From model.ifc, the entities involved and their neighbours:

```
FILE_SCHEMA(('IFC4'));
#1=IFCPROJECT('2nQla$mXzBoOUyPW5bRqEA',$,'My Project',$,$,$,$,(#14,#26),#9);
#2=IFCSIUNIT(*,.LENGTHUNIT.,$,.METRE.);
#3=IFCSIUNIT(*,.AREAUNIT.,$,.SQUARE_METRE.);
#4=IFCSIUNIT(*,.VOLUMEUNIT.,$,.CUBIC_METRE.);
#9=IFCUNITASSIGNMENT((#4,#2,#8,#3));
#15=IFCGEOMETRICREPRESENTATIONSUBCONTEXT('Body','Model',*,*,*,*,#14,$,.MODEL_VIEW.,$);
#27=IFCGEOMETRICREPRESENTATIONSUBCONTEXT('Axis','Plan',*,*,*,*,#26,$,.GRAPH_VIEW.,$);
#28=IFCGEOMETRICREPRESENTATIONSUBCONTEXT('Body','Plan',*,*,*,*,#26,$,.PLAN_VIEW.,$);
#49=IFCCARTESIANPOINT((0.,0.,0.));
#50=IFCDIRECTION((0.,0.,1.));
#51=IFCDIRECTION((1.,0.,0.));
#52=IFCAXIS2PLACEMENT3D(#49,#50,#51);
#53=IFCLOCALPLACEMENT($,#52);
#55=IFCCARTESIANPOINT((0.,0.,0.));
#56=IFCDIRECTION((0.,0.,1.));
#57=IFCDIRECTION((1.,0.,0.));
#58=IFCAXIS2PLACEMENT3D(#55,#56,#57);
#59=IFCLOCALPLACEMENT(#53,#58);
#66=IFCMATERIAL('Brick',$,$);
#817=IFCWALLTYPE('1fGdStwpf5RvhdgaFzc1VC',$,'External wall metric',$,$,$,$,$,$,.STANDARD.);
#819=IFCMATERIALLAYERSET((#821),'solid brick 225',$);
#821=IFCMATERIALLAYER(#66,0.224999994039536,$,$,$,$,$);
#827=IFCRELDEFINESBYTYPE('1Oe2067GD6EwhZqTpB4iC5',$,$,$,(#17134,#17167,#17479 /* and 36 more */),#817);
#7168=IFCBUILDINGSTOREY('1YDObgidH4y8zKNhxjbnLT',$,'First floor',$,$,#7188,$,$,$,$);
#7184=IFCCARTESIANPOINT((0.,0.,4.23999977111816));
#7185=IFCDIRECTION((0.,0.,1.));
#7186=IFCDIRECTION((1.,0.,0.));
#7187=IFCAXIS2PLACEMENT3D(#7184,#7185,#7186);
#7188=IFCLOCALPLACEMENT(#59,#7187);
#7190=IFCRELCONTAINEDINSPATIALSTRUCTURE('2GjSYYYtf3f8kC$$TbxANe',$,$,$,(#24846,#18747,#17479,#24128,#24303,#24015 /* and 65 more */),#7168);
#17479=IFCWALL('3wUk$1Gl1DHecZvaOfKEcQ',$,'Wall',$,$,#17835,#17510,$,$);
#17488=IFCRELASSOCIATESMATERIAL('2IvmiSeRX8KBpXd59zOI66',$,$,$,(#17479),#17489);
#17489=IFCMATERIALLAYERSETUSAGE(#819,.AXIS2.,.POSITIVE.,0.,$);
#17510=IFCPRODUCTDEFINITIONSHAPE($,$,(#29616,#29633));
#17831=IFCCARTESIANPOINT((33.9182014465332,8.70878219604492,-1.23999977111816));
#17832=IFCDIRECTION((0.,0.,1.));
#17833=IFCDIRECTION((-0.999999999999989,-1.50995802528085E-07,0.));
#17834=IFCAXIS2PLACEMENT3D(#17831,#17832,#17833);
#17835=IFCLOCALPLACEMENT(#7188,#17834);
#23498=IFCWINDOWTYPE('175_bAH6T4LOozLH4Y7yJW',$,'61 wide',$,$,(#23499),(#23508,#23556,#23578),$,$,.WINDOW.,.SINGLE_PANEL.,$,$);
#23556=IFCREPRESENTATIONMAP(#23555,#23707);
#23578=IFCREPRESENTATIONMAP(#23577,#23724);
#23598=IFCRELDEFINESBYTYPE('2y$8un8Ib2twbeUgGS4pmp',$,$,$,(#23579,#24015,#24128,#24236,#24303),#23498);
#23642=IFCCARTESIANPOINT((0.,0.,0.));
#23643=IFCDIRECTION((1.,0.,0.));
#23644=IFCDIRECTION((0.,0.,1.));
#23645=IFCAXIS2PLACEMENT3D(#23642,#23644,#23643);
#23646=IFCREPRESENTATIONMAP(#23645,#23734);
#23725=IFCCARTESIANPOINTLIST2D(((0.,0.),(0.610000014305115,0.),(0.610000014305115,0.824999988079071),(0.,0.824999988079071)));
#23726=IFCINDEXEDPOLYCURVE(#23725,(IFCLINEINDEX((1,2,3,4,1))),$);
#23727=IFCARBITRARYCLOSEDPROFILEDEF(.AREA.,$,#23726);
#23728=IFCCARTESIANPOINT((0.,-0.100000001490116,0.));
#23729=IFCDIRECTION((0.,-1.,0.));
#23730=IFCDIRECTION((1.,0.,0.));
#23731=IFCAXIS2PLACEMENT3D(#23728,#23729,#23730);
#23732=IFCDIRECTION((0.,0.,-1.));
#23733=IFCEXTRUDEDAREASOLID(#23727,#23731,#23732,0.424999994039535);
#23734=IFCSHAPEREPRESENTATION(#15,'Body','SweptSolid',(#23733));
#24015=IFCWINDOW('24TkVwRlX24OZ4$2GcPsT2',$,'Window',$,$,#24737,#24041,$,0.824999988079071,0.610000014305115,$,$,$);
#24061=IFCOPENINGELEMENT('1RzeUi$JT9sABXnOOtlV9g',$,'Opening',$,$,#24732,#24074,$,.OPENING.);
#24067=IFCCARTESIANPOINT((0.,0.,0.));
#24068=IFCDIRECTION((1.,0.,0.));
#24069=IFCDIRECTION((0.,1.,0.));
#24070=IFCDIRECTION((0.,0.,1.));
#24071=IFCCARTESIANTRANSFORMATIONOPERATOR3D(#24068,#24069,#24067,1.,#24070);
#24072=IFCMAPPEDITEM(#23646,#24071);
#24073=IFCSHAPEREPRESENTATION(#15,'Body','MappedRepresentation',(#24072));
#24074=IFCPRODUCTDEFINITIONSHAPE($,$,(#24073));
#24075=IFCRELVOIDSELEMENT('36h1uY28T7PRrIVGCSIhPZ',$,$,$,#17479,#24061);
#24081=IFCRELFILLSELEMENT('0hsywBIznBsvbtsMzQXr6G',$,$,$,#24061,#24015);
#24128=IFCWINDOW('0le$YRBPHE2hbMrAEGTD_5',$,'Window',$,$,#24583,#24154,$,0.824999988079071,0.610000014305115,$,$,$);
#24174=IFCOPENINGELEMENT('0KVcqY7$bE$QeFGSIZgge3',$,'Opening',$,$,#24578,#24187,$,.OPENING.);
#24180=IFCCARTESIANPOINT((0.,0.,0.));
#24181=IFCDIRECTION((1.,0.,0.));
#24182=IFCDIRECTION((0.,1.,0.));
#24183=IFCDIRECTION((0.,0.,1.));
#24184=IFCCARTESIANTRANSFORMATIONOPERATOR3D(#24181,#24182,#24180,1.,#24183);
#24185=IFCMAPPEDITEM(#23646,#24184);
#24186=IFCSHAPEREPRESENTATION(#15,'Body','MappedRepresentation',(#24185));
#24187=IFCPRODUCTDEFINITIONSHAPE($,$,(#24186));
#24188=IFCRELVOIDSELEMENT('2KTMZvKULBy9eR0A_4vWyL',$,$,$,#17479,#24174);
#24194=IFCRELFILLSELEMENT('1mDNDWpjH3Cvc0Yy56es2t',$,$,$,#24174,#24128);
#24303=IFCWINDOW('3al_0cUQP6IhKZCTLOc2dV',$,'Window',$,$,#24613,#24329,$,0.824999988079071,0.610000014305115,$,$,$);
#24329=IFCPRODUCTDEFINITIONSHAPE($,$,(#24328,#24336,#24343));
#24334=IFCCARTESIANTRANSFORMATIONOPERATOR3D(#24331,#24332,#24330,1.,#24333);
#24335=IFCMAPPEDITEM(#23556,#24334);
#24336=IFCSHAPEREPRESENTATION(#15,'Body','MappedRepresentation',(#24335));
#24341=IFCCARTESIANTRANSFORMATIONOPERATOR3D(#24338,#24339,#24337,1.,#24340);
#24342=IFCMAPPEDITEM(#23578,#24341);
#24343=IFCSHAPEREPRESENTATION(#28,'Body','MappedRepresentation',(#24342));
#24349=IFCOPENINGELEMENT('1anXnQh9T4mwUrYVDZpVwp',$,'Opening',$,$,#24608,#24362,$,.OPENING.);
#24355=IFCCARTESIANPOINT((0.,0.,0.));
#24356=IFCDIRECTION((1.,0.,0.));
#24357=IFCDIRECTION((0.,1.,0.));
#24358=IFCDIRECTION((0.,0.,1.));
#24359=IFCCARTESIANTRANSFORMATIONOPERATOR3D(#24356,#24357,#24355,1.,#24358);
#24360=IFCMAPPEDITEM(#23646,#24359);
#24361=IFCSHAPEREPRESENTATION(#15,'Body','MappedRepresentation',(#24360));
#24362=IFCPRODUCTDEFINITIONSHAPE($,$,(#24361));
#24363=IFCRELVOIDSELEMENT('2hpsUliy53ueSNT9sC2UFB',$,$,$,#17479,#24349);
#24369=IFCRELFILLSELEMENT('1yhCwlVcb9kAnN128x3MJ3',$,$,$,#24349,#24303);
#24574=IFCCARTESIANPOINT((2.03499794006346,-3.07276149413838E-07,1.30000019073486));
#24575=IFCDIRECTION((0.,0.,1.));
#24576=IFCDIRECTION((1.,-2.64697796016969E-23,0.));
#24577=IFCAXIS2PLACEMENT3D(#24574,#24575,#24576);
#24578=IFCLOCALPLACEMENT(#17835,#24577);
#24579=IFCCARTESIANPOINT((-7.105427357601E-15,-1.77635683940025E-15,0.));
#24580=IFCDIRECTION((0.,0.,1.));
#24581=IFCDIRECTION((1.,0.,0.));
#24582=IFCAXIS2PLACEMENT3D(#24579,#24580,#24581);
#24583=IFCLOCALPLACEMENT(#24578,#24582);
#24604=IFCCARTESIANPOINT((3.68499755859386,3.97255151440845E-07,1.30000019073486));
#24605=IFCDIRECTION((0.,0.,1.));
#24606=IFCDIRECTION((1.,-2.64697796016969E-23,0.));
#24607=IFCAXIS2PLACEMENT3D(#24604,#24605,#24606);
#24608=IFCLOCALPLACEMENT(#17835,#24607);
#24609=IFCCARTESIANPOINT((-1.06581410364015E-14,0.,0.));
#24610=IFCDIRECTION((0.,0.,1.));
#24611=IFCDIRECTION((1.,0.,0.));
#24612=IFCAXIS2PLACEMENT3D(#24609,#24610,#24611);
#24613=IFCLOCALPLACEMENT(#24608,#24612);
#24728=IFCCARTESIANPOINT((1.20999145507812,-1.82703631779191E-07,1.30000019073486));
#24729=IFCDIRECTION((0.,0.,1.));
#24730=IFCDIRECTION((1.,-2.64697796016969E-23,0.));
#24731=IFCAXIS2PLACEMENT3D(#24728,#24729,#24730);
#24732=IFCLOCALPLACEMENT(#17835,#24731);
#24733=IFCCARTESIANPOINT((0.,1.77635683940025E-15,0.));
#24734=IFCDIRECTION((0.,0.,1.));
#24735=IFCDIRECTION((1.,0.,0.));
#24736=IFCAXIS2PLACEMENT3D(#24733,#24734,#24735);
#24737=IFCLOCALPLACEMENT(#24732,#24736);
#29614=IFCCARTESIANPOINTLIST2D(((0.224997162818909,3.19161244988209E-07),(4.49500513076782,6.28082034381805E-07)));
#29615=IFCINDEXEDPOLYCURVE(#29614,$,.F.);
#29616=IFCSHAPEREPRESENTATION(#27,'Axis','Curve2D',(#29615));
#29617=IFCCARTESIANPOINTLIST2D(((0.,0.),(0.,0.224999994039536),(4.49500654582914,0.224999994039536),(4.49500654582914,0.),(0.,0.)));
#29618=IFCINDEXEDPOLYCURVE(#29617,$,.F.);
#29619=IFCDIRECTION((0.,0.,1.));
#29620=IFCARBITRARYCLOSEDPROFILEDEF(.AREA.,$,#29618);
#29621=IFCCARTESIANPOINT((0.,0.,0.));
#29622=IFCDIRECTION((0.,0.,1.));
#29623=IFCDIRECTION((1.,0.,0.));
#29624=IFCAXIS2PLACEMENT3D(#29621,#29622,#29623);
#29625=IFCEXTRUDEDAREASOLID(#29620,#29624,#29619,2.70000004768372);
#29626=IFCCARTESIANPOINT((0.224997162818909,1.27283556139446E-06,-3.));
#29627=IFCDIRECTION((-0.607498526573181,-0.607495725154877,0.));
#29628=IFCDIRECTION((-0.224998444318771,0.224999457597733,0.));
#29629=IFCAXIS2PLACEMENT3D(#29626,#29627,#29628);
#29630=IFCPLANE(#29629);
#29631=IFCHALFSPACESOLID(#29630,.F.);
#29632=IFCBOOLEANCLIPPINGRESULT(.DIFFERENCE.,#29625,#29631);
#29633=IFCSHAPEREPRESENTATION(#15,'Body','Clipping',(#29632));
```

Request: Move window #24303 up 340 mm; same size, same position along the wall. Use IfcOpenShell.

```python
import numpy as np
import ifcopenshell
import ifcopenshell.api.geometry
import ifcopenshell.util.placement
import ifcopenshell.util.unit

model = ifcopenshell.open("model.ifc")
unit_scale = ifcopenshell.util.unit.calculate_unit_scale(model)

window = model.by_guid("3al_0cUQP6IhKZCTLOc2dV")
opening = window.FillsVoids[0].RelatingOpeningElement
dz = 0.34 / unit_scale

shift = np.array([0.0, 0.0, dz])
# The window is placed relative to its opening, so it follows when the opening moves.
matrix = ifcopenshell.util.placement.get_local_placement(opening.ObjectPlacement)
matrix[:3, 3] += shift
ifcopenshell.api.geometry.edit_object_placement(
    model, product=opening, matrix=matrix, is_si=False, should_transform_children=True
)

print(f"moved by {dz * unit_scale:+.3f} m")

model.write("model_v2.ifc")
```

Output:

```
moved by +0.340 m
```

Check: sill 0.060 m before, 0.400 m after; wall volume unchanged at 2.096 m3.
